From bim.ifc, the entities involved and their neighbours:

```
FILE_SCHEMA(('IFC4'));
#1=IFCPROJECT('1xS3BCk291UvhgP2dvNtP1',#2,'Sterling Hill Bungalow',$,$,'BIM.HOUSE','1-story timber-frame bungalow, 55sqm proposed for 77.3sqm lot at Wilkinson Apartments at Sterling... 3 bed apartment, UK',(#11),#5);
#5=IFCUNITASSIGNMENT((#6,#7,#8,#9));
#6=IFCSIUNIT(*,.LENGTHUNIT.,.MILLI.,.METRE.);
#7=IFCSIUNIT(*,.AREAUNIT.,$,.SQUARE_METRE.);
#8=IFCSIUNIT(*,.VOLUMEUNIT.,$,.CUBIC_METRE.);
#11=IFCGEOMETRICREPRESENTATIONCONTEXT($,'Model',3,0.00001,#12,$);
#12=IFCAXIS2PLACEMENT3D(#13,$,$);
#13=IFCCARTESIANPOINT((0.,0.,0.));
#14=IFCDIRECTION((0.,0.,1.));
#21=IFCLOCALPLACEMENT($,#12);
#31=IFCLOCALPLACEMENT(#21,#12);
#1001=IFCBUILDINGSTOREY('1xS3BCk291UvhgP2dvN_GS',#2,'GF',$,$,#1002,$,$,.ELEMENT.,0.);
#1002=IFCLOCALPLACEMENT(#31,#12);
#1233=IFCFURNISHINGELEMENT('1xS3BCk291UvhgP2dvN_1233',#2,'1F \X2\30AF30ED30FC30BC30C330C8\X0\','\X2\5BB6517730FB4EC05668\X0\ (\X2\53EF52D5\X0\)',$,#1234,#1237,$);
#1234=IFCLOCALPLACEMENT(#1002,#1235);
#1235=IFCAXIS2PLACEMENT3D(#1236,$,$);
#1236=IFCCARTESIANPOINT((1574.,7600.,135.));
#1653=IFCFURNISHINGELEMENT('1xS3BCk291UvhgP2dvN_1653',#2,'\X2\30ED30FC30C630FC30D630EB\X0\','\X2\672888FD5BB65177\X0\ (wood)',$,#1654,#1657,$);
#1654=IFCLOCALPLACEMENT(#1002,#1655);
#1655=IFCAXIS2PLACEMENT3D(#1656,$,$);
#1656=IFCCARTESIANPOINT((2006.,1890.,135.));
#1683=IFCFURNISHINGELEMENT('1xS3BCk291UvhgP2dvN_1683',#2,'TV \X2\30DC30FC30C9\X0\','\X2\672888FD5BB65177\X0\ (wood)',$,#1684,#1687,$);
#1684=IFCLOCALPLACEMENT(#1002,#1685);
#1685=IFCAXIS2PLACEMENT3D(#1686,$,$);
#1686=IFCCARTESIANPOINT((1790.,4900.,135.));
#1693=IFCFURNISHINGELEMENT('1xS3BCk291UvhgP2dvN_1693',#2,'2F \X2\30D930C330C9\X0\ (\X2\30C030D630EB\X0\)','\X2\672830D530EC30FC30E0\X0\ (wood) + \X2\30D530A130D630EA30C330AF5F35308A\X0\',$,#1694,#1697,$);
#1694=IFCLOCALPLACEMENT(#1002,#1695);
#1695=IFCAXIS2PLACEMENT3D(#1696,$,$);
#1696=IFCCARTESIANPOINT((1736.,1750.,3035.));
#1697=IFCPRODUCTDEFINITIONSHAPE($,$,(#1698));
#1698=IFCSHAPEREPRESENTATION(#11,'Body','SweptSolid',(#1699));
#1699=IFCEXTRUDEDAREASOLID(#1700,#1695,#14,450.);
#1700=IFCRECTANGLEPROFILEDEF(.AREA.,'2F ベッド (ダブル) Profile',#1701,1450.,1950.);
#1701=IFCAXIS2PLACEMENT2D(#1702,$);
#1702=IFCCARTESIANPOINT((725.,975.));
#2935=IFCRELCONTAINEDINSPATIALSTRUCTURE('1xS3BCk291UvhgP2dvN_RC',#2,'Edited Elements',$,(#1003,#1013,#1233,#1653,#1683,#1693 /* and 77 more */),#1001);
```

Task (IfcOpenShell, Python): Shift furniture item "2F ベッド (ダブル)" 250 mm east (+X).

```python
import ifcopenshell
import ifcopenshell.api.geometry
import ifcopenshell.util.placement
import ifcopenshell.util.unit

model = ifcopenshell.open("bim.ifc")
unit_scale = ifcopenshell.util.unit.calculate_unit_scale(model)

item = model.by_guid("1xS3BCk291UvhgP2dvN_1693")
matrix = ifcopenshell.util.placement.get_local_placement(item.ObjectPlacement)
matrix[0, 3] += 0.25 / unit_scale
ifcopenshell.api.geometry.edit_object_placement(model, product=item, matrix=matrix, is_si=False)

print(ifcopenshell.util.placement.get_local_placement(item.ObjectPlacement).round(3) + 0.0)

model.write("bim_v2.ifc")
```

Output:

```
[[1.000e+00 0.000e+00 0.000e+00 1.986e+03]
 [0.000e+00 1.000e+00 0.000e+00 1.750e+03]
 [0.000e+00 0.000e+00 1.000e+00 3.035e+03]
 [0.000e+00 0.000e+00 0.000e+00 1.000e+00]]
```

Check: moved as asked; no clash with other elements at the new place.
